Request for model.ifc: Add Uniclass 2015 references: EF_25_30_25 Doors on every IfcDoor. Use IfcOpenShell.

First a look at what the model holds.

```python
import ifcopenshell

model = ifcopenshell.open("model.ifc")
print(model.schema)
print("classifications:", [c.Name for c in model.by_type("IfcClassification")])
for ifc_class in ("IfcDoor", "IfcRoof", "IfcStair", "IfcWall", "IfcWindow"):
    print(ifc_class, len(model.by_type(ifc_class)))
```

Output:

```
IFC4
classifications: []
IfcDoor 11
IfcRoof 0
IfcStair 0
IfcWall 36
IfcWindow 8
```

```python
import ifcopenshell
import ifcopenshell.api.classification

model = ifcopenshell.open("model.ifc")

system = ifcopenshell.api.classification.add_classification(model, classification="Uniclass 2015")

codes = {
    "IfcDoor": ("EF_25_30_25", "Doors"),
}
for ifc_class, (code, name) in codes.items():
    products = model.by_type(ifc_class)
    ifcopenshell.api.classification.add_reference(
        model, products=products, classification=system, identification=code, name=name
    )
    print(code, len(products))

model.write("model_rev.ifc")
```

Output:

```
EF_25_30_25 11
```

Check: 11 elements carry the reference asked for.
